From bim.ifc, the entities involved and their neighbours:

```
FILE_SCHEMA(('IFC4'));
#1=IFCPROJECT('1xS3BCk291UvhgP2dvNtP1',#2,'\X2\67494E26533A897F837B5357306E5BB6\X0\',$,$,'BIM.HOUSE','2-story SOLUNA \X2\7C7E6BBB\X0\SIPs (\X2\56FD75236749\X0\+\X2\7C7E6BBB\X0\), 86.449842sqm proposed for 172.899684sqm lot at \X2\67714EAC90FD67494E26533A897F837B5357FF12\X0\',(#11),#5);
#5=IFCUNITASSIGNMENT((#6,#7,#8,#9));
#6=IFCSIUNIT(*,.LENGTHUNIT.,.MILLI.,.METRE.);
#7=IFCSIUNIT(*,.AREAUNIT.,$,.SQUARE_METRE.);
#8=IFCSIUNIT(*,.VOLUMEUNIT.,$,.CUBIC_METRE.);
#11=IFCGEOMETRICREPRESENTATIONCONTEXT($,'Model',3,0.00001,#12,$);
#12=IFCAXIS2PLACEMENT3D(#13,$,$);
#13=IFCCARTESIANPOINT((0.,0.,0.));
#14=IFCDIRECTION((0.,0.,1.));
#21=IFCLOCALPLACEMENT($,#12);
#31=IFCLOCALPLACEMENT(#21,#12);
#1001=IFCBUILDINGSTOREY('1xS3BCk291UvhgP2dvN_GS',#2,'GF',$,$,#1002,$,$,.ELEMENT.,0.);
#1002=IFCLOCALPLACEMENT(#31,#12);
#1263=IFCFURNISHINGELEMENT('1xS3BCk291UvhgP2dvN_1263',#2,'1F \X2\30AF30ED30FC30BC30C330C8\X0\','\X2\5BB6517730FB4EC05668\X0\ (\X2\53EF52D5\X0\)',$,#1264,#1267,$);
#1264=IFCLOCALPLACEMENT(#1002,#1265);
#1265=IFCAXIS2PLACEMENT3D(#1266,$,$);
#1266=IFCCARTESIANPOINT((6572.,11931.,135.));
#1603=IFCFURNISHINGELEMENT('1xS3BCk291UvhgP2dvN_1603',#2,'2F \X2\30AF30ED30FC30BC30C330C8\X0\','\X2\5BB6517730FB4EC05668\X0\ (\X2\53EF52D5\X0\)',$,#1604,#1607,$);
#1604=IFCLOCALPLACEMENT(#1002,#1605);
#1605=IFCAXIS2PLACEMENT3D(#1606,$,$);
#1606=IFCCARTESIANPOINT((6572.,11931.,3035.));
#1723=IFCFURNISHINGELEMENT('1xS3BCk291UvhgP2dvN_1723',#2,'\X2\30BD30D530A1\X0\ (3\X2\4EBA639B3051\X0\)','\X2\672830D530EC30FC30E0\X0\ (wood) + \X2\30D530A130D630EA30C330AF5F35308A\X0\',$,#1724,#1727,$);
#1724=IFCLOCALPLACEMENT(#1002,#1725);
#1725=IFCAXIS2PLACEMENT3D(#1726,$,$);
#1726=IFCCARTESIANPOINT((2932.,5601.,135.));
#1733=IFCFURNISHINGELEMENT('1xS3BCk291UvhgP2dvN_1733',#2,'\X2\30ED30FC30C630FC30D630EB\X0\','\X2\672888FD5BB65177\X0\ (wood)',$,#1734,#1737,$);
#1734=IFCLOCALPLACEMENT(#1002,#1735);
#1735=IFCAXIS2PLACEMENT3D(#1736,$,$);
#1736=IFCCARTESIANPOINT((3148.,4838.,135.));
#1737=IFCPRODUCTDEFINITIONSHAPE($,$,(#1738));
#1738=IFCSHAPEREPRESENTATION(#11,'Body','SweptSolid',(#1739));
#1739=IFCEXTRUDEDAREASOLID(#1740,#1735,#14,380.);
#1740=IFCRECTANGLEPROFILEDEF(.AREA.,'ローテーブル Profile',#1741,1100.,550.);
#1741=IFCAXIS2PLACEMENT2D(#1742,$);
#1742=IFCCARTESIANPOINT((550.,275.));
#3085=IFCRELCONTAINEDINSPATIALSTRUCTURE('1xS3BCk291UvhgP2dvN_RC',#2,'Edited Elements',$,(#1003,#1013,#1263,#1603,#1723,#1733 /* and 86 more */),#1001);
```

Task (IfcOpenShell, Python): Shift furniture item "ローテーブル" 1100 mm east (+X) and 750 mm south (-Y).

```python
import ifcopenshell
import ifcopenshell.api.geometry
import ifcopenshell.util.placement

model = ifcopenshell.open("bim.ifc")

item = model.by_id(1733)
matrix = ifcopenshell.util.placement.get_local_placement(item.ObjectPlacement)
matrix[0, 3] += 1100.0
matrix[1, 3] -= 750.0
ifcopenshell.api.geometry.edit_object_placement(model, product=item, matrix=matrix, is_si=False)

print(ifcopenshell.util.placement.get_local_placement(item.ObjectPlacement).round(3) + 0.0)

model.write("bim_rev.ifc")
```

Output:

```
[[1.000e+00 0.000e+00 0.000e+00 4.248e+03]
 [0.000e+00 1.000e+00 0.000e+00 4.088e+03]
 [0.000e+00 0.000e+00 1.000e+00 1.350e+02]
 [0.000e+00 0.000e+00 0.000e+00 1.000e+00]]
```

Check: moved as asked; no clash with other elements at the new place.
